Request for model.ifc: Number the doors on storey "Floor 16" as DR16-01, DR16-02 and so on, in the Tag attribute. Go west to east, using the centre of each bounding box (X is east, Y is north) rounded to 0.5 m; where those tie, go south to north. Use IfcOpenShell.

First a look at what the model holds.

```python
import ifcopenshell
import ifcopenshell.util.element
import ifcopenshell.util.placement

model = ifcopenshell.open("model.ifc")
print(model.schema)
storey = next(s for s in model.by_type("IfcBuildingStorey") if s.Name == "Floor 16")
doors = [e for e in ifcopenshell.util.element.get_decomposition(storey) if e.is_a("IfcDoor")]
for e in sorted(doors, key=lambda e: e.id()):
    origin = ifcopenshell.util.placement.get_local_placement(e.ObjectPlacement)[:3, 3]
    print(e.id(), e.Tag, e.Name, origin.round(2) + 0.0, sep=" | ")
```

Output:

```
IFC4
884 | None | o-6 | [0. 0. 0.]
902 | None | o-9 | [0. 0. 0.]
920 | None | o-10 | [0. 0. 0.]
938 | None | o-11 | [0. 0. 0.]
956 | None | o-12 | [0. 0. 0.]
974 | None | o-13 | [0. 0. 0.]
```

```python
import ifcopenshell
import ifcopenshell.geom
import ifcopenshell.util.element
import ifcopenshell.util.shape

model = ifcopenshell.open("model.ifc")
settings = ifcopenshell.geom.settings()
settings.set("use-world-coords", True)


def centre(element):
    shape = ifcopenshell.geom.create_shape(settings, element)
    return ifcopenshell.util.shape.get_bbox_centroid(shape.geometry)


storey = next(s for s in model.by_type("IfcBuildingStorey") if s.Name == "Floor 16")
doors = [e for e in ifcopenshell.util.element.get_decomposition(storey) if e.is_a("IfcDoor")]

# Insertion points can sit at a corner or the storey origin, so sort by the geometry (in metres).
centres = {e: centre(e) for e in doors}
doors.sort(key=lambda e: (round(centres[e][0] / 0.5), centres[e][1]))

for i, e in enumerate(doors, start=1):
    number = f"DR16-{i:02d}"
    e.Tag = number
    print(e.id(), number)

model.write("model-out.ifc")
```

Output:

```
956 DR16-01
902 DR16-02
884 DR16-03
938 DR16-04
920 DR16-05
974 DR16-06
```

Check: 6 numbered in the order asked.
